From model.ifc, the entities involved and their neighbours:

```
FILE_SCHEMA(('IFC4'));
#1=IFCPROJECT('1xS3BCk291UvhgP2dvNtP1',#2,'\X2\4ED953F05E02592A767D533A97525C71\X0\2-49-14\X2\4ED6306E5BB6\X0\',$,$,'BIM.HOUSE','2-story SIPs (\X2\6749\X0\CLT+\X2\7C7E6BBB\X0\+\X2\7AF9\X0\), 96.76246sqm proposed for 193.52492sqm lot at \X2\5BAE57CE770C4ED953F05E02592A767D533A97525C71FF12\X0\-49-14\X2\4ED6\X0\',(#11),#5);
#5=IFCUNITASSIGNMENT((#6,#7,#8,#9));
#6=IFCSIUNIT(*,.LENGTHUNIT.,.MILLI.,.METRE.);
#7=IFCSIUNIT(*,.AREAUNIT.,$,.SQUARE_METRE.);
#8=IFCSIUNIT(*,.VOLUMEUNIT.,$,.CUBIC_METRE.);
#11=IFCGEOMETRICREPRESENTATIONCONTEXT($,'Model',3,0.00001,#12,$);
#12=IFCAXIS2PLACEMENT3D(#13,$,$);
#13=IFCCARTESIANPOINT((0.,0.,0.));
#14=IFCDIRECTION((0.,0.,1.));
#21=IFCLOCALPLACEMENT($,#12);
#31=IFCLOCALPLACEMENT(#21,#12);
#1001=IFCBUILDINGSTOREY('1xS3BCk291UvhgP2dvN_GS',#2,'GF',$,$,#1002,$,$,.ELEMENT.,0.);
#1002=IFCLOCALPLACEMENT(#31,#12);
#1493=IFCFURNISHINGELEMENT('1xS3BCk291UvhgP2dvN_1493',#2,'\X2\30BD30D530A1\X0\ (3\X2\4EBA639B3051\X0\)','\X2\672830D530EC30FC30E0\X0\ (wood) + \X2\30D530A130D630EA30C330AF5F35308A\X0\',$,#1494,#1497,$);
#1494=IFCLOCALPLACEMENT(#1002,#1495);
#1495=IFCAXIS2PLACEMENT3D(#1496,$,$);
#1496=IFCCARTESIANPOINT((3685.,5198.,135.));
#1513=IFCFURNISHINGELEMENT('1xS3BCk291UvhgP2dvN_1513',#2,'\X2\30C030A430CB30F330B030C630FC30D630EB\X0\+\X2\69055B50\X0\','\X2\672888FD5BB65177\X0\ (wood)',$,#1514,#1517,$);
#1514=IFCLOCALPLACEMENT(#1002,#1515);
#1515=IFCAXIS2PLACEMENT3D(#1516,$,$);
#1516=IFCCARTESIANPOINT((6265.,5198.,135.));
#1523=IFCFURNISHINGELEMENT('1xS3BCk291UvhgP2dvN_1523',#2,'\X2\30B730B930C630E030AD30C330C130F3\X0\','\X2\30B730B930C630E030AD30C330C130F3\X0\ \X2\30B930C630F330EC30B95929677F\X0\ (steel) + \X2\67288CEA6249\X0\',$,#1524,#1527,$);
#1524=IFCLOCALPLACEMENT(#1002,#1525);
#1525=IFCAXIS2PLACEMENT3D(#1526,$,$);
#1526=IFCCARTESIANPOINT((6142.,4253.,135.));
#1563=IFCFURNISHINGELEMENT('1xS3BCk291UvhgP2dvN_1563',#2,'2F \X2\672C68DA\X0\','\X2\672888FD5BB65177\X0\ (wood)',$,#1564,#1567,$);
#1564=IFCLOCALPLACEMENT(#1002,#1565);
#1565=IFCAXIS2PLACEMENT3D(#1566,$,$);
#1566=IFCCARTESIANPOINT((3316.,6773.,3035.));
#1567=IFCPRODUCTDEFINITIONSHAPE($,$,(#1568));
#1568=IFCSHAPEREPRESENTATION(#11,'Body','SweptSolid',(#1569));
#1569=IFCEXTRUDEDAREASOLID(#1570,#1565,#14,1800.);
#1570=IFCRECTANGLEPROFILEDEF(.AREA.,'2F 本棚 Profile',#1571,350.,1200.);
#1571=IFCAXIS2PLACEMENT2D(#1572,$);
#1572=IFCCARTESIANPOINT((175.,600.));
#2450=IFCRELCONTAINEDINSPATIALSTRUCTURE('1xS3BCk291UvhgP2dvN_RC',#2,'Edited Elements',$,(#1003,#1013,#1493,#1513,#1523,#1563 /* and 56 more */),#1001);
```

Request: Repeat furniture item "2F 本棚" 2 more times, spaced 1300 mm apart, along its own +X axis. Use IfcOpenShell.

```python
import ifcopenshell
import ifcopenshell.api.geometry
import ifcopenshell.api.root
import ifcopenshell.util.element
import ifcopenshell.util.placement
import ifcopenshell.util.unit

model = ifcopenshell.open("model.ifc")
unit_scale = ifcopenshell.util.unit.calculate_unit_scale(model)


def reuse_history(source, copy):
    """copy_class also copies each property set's owner history, people and application; keep the originals."""
    for rel in copy.IsDefinedBy:
        if rel.is_a("IfcRelDefinesByProperties") and (history := rel.RelatingPropertyDefinition.OwnerHistory):
            rel.RelatingPropertyDefinition.OwnerHistory = source.OwnerHistory
            ifcopenshell.util.element.remove_deep2(model, history)


source = model.by_id(1563)
base = ifcopenshell.util.placement.get_local_placement(source.ObjectPlacement)
step = base[:3, 0] * 1.3 / unit_scale

for i in range(1, 3):
    copy = ifcopenshell.api.root.copy_class(model, product=source)
    copy.Representation = ifcopenshell.util.element.copy_deep(
        model, source.Representation, exclude=["IfcGeometricRepresentationContext", "IfcRepresentationMap"]
    )
    reuse_history(source, copy)
    matrix = base.copy()
    matrix[:3, 3] += i * step
    print("added at", matrix[:3, 3].round(3) + 0.0)
    ifcopenshell.api.geometry.edit_object_placement(model, product=copy, matrix=matrix, is_si=False)

model.write("model-out.ifc")
```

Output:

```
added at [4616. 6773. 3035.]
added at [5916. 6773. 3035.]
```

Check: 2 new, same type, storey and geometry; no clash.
